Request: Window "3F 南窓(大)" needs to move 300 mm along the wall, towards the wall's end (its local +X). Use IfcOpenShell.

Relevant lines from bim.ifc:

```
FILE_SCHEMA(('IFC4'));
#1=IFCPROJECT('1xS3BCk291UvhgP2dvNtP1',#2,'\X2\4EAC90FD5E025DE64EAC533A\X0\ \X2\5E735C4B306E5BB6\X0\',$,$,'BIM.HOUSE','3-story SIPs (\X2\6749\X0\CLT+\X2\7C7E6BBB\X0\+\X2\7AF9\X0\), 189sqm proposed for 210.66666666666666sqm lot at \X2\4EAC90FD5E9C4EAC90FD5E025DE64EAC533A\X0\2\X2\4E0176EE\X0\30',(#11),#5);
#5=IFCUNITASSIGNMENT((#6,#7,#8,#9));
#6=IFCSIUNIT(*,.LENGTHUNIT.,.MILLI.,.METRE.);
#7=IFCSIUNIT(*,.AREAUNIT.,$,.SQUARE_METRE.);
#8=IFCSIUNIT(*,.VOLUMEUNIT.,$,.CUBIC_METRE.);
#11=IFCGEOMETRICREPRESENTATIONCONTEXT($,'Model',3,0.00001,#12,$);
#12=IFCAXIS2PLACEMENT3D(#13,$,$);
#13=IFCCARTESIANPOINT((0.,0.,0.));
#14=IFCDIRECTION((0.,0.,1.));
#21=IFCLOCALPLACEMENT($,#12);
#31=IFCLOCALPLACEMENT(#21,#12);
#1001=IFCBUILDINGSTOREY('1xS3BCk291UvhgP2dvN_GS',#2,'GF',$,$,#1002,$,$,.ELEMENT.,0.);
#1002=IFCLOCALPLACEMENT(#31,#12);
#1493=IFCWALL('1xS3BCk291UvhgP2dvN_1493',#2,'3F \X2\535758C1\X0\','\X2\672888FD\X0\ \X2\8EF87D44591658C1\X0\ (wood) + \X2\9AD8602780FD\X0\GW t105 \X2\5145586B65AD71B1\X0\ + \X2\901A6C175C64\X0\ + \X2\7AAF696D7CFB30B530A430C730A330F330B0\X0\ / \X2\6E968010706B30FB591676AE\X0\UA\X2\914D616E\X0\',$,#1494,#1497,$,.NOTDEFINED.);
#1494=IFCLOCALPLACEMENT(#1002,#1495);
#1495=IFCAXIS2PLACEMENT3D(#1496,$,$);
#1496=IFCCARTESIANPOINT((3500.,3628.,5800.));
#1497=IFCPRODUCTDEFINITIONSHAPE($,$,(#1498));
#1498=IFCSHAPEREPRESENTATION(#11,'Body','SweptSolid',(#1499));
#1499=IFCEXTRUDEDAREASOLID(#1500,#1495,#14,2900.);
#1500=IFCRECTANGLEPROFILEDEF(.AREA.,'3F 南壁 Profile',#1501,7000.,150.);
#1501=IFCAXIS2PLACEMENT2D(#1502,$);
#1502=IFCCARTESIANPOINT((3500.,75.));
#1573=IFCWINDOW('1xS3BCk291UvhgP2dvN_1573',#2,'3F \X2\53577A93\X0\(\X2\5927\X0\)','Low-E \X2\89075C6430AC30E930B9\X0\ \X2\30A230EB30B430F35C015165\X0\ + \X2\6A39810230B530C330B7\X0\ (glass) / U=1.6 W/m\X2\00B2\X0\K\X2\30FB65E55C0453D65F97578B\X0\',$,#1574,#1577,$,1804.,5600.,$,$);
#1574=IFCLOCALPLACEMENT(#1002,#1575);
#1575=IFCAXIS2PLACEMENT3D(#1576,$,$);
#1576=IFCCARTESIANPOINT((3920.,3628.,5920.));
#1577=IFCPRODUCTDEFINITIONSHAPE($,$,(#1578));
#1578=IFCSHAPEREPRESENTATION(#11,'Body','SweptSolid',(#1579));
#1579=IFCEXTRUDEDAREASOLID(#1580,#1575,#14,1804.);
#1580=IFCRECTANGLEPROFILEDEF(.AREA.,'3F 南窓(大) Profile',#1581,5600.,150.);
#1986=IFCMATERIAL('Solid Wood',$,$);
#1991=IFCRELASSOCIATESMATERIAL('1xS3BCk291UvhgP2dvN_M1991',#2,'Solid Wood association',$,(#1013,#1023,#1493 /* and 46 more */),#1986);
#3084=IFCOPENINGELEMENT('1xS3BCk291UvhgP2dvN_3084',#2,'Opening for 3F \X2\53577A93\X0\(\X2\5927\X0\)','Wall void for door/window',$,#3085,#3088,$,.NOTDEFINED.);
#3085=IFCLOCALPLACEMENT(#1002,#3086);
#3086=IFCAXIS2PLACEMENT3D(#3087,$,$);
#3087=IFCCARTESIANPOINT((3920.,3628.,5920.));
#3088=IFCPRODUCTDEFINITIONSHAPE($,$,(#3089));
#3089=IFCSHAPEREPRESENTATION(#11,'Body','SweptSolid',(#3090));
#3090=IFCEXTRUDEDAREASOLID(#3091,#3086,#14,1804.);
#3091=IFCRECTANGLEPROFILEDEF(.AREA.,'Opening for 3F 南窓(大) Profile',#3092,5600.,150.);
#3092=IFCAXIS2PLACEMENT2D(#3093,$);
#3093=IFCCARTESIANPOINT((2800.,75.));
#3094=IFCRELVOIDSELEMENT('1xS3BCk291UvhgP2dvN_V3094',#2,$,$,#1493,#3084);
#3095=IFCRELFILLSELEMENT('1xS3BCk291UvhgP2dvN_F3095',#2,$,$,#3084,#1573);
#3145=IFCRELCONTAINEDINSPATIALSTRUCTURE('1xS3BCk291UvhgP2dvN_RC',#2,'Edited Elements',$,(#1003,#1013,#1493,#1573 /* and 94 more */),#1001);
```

```python
import ifcopenshell
import ifcopenshell.api.geometry
import ifcopenshell.util.placement
import ifcopenshell.util.unit

model = ifcopenshell.open("bim.ifc")
unit_scale = ifcopenshell.util.unit.calculate_unit_scale(model)

window = model.by_id(1573)
opening = window.FillsVoids[0].RelatingOpeningElement
wall = opening.VoidsElements[0].RelatingBuildingElement

wall_matrix = ifcopenshell.util.placement.get_local_placement(wall.ObjectPlacement)
shift = wall_matrix[:3, 0] * 0.3 / unit_scale
before = ifcopenshell.util.placement.get_local_placement(window.ObjectPlacement)[:3, 3].copy()

# The window is not placed relative to its opening, so move both.
for product in (opening, window):
    matrix = ifcopenshell.util.placement.get_local_placement(product.ObjectPlacement)
    matrix[:3, 3] += shift
    ifcopenshell.api.geometry.edit_object_placement(model, product=product, matrix=matrix, is_si=False)

after = ifcopenshell.util.placement.get_local_placement(window.ObjectPlacement)[:3, 3]
print("window moved by", (after - before).round(3) + 0.0)

model.write("bim_v2.ifc")
```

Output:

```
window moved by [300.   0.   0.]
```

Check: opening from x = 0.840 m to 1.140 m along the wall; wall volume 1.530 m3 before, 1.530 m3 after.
